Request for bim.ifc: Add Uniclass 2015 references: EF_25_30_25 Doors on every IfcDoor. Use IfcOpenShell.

First a look at what the model holds.

```python
import ifcopenshell

model = ifcopenshell.open("bim.ifc")
print(model.schema)
print("classifications:", [c.Name for c in model.by_type("IfcClassification")])
for ifc_class in ("IfcDoor", "IfcRoof", "IfcStair", "IfcWall", "IfcWindow"):
    print(ifc_class, len(model.by_type(ifc_class)))
```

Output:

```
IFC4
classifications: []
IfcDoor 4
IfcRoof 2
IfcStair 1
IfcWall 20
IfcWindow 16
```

```python
import ifcopenshell
import ifcopenshell.api.classification

model = ifcopenshell.open("bim.ifc")

system = ifcopenshell.api.classification.add_classification(model, classification="Uniclass 2015")

codes = {
    "IfcDoor": ("EF_25_30_25", "Doors"),
}
for ifc_class, (code, name) in codes.items():
    products = model.by_type(ifc_class)
    ifcopenshell.api.classification.add_reference(
        model, products=products, classification=system, identification=code, name=name
    )
    print(code, len(products))

model.write("bim_rev.ifc")
```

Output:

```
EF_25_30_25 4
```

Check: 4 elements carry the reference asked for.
